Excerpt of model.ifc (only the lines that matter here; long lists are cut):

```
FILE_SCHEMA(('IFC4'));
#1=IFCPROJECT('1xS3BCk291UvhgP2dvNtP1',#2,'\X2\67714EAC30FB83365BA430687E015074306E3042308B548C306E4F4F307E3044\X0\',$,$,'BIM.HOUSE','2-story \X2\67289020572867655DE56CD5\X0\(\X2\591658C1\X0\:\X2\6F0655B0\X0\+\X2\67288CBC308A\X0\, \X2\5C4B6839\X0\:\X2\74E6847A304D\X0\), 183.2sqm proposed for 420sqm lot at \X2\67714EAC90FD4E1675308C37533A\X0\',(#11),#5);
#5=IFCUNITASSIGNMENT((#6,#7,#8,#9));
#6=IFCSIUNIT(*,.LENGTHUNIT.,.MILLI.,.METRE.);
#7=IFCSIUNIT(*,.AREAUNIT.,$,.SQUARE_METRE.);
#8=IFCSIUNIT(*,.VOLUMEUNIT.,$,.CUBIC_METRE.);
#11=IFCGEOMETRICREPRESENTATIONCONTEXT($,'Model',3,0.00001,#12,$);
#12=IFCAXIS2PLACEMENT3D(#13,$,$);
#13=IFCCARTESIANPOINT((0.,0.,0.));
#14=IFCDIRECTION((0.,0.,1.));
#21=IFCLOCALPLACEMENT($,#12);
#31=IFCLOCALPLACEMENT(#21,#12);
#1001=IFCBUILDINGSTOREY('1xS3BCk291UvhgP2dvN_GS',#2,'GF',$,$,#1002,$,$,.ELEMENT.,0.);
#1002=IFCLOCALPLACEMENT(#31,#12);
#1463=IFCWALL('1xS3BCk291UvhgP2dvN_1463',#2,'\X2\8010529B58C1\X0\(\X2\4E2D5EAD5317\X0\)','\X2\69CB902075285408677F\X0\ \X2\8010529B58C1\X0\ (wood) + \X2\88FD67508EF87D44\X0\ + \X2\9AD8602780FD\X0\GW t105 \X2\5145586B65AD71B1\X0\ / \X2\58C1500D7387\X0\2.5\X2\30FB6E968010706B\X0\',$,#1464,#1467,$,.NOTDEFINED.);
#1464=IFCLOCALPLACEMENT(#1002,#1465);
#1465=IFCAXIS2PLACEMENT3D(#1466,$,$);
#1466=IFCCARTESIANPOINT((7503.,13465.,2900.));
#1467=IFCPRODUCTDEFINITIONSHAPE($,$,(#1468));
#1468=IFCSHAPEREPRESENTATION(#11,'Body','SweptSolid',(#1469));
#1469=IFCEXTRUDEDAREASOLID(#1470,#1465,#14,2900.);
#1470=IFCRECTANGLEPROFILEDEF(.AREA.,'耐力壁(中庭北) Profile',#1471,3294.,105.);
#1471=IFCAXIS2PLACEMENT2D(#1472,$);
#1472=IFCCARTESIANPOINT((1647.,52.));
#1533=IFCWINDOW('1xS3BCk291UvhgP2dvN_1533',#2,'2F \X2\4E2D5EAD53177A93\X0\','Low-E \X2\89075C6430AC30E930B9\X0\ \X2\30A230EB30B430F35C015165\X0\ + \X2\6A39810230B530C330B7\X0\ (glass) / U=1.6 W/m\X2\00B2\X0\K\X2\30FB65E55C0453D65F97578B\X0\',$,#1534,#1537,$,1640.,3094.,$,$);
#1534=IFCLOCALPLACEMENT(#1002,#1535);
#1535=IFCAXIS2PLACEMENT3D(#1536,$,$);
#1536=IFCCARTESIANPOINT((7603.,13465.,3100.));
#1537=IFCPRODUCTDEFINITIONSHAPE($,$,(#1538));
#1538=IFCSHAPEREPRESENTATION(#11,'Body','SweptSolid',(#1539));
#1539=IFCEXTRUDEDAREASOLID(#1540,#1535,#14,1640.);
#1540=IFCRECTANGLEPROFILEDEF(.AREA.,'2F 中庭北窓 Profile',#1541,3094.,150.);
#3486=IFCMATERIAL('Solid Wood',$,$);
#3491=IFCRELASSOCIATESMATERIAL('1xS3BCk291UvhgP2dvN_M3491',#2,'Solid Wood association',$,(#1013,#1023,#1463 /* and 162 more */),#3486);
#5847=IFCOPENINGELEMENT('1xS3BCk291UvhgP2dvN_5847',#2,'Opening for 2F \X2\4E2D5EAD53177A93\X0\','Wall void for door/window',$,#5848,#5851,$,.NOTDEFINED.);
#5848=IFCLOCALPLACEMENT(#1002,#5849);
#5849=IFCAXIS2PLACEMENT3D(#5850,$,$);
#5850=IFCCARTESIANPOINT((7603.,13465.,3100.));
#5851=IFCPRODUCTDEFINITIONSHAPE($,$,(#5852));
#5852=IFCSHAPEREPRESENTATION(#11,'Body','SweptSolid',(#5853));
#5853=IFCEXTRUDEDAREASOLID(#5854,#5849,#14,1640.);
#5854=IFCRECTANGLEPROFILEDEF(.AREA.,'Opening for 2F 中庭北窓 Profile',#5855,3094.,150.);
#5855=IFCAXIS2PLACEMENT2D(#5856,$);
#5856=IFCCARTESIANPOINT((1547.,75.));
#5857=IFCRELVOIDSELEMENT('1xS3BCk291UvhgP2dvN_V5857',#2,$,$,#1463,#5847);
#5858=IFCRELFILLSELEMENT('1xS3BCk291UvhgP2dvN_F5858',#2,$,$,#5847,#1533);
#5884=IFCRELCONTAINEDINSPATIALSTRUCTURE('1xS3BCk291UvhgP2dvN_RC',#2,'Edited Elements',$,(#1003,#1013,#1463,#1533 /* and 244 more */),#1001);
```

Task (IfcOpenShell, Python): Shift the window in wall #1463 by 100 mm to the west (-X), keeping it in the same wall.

```python
import ifcopenshell
import ifcopenshell.api.geometry
import ifcopenshell.util.placement
import ifcopenshell.util.unit

model = ifcopenshell.open("model.ifc")
unit_scale = ifcopenshell.util.unit.calculate_unit_scale(model)

window = model.by_guid("1xS3BCk291UvhgP2dvN_1533")
opening = window.FillsVoids[0].RelatingOpeningElement
wall = opening.VoidsElements[0].RelatingBuildingElement

wall_matrix = ifcopenshell.util.placement.get_local_placement(wall.ObjectPlacement)
shift = wall_matrix[:3, 0] * -0.1 / unit_scale
before = ifcopenshell.util.placement.get_local_placement(window.ObjectPlacement)[:3, 3].copy()

# The window is not placed relative to its opening, so move both.
for product in (opening, window):
    matrix = ifcopenshell.util.placement.get_local_placement(product.ObjectPlacement)
    matrix[:3, 3] += shift
    ifcopenshell.api.geometry.edit_object_placement(model, product=product, matrix=matrix, is_si=False)

after = ifcopenshell.util.placement.get_local_placement(window.ObjectPlacement)[:3, 3]
print("window moved by", (after - before).round(3) + 0.0)

model.write("model_v2.ifc")
```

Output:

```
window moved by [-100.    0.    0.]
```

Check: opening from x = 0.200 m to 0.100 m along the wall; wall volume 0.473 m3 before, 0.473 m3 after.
